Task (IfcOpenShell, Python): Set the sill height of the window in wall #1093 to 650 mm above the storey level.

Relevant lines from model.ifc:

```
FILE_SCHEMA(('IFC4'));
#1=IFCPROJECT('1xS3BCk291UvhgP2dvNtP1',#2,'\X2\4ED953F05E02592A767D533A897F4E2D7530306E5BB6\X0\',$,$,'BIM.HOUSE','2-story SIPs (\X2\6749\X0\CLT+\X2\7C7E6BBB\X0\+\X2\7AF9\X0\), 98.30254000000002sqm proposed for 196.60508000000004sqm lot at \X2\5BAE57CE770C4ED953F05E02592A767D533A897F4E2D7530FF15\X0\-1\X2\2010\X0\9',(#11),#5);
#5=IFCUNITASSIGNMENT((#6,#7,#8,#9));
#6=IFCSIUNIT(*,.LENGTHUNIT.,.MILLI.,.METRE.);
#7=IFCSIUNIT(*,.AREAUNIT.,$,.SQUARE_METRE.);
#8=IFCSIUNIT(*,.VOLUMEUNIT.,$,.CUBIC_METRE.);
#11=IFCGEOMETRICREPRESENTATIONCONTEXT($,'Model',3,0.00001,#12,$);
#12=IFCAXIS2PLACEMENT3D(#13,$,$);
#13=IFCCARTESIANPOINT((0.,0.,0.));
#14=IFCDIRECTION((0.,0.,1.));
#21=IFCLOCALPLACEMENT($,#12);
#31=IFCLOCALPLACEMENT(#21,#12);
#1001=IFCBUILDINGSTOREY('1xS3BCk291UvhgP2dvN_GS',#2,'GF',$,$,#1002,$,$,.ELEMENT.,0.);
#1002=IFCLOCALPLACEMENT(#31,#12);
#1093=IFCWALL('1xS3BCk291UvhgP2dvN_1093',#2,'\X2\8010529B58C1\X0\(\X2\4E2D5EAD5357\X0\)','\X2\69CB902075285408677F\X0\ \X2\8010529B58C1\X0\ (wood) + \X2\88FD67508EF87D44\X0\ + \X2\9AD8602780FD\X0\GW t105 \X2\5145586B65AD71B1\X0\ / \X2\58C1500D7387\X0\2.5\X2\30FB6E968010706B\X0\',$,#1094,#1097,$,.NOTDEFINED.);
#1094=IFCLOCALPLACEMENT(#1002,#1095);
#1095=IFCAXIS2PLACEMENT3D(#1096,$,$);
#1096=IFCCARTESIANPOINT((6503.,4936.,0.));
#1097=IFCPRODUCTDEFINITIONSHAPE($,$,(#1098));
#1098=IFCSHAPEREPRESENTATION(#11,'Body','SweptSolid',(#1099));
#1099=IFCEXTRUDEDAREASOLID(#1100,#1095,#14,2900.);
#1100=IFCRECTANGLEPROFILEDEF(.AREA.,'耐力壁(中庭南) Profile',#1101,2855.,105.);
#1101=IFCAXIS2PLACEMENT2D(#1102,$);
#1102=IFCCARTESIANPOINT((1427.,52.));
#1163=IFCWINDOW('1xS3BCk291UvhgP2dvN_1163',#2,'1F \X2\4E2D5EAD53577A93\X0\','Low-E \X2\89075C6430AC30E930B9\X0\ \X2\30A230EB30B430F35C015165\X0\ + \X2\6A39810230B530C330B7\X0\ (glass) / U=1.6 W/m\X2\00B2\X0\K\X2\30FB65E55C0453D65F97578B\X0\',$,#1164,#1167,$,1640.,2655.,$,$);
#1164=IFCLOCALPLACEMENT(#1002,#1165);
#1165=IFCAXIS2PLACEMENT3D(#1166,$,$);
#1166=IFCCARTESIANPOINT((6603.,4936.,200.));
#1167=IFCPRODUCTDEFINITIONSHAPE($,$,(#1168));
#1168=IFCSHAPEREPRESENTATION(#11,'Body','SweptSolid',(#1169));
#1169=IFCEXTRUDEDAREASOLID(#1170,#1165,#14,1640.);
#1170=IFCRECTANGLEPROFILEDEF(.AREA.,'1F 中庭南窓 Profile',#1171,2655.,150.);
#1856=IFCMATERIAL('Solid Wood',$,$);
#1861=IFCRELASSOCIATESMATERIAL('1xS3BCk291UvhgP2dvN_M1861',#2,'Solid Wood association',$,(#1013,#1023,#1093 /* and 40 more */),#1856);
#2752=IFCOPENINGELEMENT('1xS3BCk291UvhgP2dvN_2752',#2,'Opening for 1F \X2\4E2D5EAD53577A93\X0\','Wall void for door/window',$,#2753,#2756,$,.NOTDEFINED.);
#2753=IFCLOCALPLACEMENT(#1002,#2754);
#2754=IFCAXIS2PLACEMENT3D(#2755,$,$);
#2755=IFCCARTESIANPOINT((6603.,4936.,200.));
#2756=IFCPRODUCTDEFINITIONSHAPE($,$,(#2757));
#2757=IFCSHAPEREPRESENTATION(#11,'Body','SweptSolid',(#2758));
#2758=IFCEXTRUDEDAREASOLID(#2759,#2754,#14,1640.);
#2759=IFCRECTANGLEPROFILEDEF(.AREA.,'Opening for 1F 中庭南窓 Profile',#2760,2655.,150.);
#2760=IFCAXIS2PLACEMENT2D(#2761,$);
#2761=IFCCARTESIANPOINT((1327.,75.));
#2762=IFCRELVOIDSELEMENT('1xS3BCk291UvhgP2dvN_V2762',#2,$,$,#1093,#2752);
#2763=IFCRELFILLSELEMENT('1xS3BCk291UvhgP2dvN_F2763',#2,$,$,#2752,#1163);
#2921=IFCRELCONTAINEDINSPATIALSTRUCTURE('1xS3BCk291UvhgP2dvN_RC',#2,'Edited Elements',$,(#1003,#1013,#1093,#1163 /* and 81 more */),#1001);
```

```python
import numpy as np
import ifcopenshell
import ifcopenshell.api.geometry
import ifcopenshell.geom
import ifcopenshell.util.element
import ifcopenshell.util.placement
import ifcopenshell.util.shape
import ifcopenshell.util.unit

model = ifcopenshell.open("model.ifc")
unit_scale = ifcopenshell.util.unit.calculate_unit_scale(model)

window = model.by_guid("1xS3BCk291UvhgP2dvN_1163")
opening = window.FillsVoids[0].RelatingOpeningElement
storey = ifcopenshell.util.element.get_container(window, ifc_class="IfcBuildingStorey")
level = ifcopenshell.util.placement.get_local_placement(storey.ObjectPlacement)[2, 3]

# The opening's origin need not be at the sill, so measure its lowest point.
shape = ifcopenshell.geom.create_shape(ifcopenshell.geom.settings(), opening)
bottom = ifcopenshell.util.shape.get_shape_bottom_elevation(shape, shape.geometry) / unit_scale
dz = level + 0.65 / unit_scale - bottom

shift = np.array([0.0, 0.0, dz])
# The window is not placed relative to its opening, so move both.
for product in (opening, window):
    matrix = ifcopenshell.util.placement.get_local_placement(product.ObjectPlacement)
    matrix[:3, 3] += shift
    ifcopenshell.api.geometry.edit_object_placement(model, product=product, matrix=matrix, is_si=False)

print(f"moved by {dz * unit_scale:+.3f} m")

model.write("model-out.ifc")
```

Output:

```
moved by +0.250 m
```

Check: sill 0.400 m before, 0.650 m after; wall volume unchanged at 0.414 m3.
